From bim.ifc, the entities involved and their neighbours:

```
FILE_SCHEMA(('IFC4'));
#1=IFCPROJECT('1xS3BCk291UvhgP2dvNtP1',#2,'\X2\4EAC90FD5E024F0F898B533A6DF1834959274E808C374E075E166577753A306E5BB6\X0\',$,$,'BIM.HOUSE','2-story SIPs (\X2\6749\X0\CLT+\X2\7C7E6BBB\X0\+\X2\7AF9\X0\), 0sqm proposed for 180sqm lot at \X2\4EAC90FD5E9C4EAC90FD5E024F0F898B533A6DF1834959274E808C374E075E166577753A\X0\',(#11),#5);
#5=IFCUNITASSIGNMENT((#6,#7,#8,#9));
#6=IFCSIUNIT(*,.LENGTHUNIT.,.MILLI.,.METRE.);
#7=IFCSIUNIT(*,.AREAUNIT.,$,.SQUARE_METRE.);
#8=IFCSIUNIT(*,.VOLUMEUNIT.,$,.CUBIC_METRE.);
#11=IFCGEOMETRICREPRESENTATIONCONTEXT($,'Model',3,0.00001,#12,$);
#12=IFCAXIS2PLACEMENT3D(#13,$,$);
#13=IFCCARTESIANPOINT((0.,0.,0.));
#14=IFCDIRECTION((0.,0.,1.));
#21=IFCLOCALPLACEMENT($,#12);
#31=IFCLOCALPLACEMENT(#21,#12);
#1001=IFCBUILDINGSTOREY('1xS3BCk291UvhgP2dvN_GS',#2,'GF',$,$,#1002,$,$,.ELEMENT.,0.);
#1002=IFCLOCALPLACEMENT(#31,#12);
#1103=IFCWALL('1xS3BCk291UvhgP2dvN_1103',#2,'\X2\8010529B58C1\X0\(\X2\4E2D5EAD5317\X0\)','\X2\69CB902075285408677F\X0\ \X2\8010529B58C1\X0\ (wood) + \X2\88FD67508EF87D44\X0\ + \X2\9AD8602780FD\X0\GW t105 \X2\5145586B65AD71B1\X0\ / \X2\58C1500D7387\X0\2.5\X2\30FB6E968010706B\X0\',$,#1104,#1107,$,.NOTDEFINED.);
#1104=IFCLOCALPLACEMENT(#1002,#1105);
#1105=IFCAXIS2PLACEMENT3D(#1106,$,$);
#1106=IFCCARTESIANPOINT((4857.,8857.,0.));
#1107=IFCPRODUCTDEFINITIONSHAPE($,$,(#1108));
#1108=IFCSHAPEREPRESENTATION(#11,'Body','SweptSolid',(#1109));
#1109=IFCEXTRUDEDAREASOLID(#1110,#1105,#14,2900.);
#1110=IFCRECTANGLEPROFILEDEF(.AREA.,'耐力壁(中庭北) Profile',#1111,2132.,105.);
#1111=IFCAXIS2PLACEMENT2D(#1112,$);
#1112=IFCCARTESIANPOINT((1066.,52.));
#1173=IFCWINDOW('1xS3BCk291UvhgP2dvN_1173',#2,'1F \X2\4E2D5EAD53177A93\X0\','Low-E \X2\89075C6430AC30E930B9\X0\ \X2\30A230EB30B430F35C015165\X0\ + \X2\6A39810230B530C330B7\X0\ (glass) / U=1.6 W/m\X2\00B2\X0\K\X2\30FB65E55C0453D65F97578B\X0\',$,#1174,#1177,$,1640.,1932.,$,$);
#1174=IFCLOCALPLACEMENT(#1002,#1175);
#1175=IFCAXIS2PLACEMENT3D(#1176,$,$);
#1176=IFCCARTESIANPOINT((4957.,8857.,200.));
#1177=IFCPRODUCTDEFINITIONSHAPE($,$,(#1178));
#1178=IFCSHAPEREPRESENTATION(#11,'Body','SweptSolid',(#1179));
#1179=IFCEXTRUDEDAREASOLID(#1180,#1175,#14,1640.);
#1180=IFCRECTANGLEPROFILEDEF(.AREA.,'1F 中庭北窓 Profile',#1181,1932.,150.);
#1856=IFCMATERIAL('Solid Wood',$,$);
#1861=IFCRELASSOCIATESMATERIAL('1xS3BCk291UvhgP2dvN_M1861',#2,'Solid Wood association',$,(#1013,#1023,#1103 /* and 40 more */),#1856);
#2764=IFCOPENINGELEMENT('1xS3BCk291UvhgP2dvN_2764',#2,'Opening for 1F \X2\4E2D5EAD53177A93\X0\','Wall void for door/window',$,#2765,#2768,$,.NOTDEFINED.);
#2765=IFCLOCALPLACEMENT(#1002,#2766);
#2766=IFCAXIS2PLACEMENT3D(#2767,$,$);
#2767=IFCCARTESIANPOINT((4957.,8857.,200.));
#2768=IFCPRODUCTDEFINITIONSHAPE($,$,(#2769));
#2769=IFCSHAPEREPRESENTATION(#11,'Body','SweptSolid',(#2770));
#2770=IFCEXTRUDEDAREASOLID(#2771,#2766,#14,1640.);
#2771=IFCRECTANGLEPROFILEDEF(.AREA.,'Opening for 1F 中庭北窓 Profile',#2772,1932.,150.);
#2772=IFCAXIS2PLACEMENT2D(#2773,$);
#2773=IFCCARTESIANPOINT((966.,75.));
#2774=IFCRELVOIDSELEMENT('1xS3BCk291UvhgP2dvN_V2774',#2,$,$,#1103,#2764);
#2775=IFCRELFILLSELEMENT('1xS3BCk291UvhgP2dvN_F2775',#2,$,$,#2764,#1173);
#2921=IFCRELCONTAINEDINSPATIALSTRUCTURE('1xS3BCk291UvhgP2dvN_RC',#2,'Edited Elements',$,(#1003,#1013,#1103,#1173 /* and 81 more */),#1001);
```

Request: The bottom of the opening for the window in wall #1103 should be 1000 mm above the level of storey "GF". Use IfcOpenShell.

```python
import numpy as np
import ifcopenshell
import ifcopenshell.api.geometry
import ifcopenshell.geom
import ifcopenshell.util.element
import ifcopenshell.util.placement
import ifcopenshell.util.shape
import ifcopenshell.util.unit

model = ifcopenshell.open("bim.ifc")
unit_scale = ifcopenshell.util.unit.calculate_unit_scale(model)

window = model.by_id(1173)
opening = window.FillsVoids[0].RelatingOpeningElement
storey = ifcopenshell.util.element.get_container(window, ifc_class="IfcBuildingStorey")
level = ifcopenshell.util.placement.get_local_placement(storey.ObjectPlacement)[2, 3]

# The opening's origin need not be at the sill, so measure its lowest point.
shape = ifcopenshell.geom.create_shape(ifcopenshell.geom.settings(), opening)
bottom = ifcopenshell.util.shape.get_shape_bottom_elevation(shape, shape.geometry) / unit_scale
dz = level + 1000.0 - bottom

shift = np.array([0.0, 0.0, dz])
# The window is not placed relative to its opening, so move both.
for product in (opening, window):
    matrix = ifcopenshell.util.placement.get_local_placement(product.ObjectPlacement)
    matrix[:3, 3] += shift
    ifcopenshell.api.geometry.edit_object_placement(model, product=product, matrix=matrix, is_si=False)

print(f"moved by {dz * unit_scale:+.3f} m")

model.write("bim_rev.ifc")
```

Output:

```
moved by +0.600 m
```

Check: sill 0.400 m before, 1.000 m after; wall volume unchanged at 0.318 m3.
